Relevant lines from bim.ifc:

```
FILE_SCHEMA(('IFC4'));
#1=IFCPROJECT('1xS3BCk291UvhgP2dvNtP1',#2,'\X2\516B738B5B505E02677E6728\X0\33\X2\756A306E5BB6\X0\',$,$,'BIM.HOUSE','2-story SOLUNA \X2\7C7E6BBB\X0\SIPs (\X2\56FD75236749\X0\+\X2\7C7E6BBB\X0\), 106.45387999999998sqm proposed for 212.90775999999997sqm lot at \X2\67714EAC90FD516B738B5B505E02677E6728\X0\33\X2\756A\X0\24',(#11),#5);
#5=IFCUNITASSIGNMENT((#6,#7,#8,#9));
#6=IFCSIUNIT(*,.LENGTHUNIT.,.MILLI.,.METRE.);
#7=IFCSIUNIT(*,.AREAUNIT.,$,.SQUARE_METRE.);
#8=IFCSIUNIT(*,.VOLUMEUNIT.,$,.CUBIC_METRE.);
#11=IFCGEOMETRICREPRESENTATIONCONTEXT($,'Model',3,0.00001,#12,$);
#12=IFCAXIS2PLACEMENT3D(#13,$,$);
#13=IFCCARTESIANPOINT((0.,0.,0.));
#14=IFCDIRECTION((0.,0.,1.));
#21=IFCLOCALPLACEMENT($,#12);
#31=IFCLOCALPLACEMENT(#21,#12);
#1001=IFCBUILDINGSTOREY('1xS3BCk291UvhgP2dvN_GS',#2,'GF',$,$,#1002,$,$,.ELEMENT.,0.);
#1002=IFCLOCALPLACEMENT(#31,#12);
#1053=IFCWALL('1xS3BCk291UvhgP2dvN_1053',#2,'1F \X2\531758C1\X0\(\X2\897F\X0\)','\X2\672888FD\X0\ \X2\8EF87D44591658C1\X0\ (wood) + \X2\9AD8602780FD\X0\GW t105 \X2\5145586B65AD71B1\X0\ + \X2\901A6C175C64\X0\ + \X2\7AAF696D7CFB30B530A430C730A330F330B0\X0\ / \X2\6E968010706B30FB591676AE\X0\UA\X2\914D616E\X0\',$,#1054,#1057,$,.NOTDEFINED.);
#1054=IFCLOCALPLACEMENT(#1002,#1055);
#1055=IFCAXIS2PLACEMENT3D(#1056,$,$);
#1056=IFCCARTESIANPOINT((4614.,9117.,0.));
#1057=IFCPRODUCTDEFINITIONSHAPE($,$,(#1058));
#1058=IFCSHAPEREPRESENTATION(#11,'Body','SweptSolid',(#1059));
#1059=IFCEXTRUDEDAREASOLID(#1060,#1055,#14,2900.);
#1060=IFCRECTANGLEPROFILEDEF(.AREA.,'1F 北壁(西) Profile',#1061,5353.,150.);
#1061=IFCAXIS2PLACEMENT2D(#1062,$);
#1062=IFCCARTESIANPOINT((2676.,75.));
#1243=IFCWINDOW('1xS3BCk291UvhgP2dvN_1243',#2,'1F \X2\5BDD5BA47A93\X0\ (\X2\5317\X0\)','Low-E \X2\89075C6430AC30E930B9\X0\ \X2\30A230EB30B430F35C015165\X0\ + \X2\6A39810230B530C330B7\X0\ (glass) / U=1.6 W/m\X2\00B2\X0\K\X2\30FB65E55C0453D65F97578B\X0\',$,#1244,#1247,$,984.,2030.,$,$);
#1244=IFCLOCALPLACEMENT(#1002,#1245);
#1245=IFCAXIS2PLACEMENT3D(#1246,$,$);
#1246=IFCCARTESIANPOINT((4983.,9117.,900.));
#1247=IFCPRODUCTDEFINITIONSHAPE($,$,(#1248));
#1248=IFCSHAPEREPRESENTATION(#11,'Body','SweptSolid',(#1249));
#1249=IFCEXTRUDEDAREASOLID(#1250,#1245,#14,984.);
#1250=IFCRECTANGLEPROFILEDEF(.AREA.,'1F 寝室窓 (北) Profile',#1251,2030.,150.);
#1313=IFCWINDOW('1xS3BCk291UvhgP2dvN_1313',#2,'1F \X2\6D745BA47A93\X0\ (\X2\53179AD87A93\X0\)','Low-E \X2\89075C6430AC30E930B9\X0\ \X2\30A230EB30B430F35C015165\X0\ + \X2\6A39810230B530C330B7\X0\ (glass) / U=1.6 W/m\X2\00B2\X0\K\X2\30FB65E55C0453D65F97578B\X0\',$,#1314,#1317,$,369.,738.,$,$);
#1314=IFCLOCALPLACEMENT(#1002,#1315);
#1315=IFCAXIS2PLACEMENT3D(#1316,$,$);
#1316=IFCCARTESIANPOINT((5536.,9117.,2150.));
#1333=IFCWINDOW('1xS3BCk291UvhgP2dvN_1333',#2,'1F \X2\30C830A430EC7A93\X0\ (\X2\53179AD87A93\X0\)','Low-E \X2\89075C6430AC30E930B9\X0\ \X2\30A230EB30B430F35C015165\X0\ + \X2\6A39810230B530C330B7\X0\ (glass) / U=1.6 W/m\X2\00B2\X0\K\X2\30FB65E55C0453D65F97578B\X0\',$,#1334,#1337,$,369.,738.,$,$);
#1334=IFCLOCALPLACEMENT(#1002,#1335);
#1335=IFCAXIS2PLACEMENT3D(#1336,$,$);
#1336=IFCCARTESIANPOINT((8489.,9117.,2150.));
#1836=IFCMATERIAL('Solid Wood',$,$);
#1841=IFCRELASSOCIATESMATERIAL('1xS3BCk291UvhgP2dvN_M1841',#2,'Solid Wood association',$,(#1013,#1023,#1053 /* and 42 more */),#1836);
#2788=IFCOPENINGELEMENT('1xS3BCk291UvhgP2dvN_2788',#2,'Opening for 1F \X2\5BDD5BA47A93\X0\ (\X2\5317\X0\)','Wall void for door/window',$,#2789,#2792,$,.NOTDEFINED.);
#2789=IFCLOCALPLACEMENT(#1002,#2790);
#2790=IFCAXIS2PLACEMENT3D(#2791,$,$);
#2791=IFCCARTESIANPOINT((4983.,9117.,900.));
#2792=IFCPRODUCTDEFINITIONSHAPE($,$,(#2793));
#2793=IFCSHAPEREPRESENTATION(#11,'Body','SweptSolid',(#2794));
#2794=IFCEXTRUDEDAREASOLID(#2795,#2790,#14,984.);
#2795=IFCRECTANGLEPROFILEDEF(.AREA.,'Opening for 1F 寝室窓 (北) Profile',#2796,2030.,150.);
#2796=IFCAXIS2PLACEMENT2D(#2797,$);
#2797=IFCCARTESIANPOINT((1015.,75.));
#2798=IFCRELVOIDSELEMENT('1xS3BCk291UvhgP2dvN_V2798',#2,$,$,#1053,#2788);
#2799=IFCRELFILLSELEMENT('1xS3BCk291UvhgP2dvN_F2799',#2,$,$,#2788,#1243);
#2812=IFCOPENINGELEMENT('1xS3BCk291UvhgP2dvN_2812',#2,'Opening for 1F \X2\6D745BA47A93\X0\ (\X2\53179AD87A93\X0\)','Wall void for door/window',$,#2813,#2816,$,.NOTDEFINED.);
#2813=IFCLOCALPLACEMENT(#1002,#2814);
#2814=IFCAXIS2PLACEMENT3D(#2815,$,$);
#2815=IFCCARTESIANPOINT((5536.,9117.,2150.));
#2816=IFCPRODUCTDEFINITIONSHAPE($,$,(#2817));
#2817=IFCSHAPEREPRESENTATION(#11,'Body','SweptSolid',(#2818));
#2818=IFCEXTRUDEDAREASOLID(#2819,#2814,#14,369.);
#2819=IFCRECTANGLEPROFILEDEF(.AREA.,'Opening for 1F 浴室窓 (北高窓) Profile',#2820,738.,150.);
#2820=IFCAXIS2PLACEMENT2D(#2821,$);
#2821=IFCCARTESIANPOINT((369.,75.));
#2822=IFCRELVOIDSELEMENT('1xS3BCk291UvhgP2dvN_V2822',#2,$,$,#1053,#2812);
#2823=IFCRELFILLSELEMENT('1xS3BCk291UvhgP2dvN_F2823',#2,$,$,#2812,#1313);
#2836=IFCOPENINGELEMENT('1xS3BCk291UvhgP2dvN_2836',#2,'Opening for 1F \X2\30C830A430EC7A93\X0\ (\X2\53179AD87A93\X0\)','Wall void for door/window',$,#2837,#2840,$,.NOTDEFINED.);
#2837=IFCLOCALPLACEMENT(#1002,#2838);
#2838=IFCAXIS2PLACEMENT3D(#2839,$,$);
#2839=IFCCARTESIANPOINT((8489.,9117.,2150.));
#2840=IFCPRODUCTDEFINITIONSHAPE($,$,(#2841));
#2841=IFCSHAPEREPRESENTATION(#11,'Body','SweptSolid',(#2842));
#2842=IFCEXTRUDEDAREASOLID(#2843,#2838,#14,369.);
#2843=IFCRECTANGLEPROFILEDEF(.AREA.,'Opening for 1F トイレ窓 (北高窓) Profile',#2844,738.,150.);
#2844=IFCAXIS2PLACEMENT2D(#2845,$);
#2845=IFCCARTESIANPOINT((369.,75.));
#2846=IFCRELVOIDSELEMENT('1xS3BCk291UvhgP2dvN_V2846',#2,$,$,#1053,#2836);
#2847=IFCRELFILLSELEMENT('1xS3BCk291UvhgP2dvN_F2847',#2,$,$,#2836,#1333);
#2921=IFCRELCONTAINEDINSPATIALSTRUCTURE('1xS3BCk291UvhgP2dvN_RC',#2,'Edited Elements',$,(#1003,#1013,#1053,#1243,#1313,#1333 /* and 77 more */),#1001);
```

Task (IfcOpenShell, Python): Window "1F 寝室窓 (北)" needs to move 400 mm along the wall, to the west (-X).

```python
import ifcopenshell
import ifcopenshell.api.geometry
import ifcopenshell.util.placement

model = ifcopenshell.open("bim.ifc")

window = model.by_guid("1xS3BCk291UvhgP2dvN_1243")
opening = window.FillsVoids[0].RelatingOpeningElement
wall = opening.VoidsElements[0].RelatingBuildingElement

wall_matrix = ifcopenshell.util.placement.get_local_placement(wall.ObjectPlacement)
shift = wall_matrix[:3, 0] * -400.0
before = ifcopenshell.util.placement.get_local_placement(window.ObjectPlacement)[:3, 3].copy()

# The window is not placed relative to its opening, so move both.
for product in (opening, window):
    matrix = ifcopenshell.util.placement.get_local_placement(product.ObjectPlacement)
    matrix[:3, 3] += shift
    ifcopenshell.api.geometry.edit_object_placement(model, product=product, matrix=matrix, is_si=False)

after = ifcopenshell.util.placement.get_local_placement(window.ObjectPlacement)[:3, 3]
print("window moved by", (after - before).round(3) + 0.0)

model.write("bim_v2.ifc")
```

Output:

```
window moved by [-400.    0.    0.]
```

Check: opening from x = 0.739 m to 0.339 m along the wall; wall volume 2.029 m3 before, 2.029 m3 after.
